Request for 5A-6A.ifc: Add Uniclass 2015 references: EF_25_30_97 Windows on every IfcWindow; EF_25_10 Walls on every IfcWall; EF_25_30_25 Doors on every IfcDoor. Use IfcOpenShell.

First a look at what the model holds.

```python
import ifcopenshell

model = ifcopenshell.open("5A-6A.ifc")
print(model.schema)
print("classifications:", [c.Name for c in model.by_type("IfcClassification")])
for ifc_class in ("IfcDoor", "IfcRoof", "IfcStair", "IfcWall", "IfcWindow"):
    print(ifc_class, len(model.by_type(ifc_class)))
```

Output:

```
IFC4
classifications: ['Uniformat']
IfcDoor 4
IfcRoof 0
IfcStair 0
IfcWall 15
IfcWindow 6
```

```python
import ifcopenshell
import ifcopenshell.api.classification

model = ifcopenshell.open("5A-6A.ifc")

system = ifcopenshell.api.classification.add_classification(model, classification="Uniclass 2015")

codes = {
    "IfcWindow": ("EF_25_30_97", "Windows"),
    "IfcWall": ("EF_25_10", "Walls"),
    "IfcDoor": ("EF_25_30_25", "Doors"),
}
for ifc_class, (code, name) in codes.items():
    products = model.by_type(ifc_class)
    ifcopenshell.api.classification.add_reference(
        model, products=products, classification=system, identification=code, name=name
    )
    print(code, len(products))

model.write("5A-6A_v2.ifc")
```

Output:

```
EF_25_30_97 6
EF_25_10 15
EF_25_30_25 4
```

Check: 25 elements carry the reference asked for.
